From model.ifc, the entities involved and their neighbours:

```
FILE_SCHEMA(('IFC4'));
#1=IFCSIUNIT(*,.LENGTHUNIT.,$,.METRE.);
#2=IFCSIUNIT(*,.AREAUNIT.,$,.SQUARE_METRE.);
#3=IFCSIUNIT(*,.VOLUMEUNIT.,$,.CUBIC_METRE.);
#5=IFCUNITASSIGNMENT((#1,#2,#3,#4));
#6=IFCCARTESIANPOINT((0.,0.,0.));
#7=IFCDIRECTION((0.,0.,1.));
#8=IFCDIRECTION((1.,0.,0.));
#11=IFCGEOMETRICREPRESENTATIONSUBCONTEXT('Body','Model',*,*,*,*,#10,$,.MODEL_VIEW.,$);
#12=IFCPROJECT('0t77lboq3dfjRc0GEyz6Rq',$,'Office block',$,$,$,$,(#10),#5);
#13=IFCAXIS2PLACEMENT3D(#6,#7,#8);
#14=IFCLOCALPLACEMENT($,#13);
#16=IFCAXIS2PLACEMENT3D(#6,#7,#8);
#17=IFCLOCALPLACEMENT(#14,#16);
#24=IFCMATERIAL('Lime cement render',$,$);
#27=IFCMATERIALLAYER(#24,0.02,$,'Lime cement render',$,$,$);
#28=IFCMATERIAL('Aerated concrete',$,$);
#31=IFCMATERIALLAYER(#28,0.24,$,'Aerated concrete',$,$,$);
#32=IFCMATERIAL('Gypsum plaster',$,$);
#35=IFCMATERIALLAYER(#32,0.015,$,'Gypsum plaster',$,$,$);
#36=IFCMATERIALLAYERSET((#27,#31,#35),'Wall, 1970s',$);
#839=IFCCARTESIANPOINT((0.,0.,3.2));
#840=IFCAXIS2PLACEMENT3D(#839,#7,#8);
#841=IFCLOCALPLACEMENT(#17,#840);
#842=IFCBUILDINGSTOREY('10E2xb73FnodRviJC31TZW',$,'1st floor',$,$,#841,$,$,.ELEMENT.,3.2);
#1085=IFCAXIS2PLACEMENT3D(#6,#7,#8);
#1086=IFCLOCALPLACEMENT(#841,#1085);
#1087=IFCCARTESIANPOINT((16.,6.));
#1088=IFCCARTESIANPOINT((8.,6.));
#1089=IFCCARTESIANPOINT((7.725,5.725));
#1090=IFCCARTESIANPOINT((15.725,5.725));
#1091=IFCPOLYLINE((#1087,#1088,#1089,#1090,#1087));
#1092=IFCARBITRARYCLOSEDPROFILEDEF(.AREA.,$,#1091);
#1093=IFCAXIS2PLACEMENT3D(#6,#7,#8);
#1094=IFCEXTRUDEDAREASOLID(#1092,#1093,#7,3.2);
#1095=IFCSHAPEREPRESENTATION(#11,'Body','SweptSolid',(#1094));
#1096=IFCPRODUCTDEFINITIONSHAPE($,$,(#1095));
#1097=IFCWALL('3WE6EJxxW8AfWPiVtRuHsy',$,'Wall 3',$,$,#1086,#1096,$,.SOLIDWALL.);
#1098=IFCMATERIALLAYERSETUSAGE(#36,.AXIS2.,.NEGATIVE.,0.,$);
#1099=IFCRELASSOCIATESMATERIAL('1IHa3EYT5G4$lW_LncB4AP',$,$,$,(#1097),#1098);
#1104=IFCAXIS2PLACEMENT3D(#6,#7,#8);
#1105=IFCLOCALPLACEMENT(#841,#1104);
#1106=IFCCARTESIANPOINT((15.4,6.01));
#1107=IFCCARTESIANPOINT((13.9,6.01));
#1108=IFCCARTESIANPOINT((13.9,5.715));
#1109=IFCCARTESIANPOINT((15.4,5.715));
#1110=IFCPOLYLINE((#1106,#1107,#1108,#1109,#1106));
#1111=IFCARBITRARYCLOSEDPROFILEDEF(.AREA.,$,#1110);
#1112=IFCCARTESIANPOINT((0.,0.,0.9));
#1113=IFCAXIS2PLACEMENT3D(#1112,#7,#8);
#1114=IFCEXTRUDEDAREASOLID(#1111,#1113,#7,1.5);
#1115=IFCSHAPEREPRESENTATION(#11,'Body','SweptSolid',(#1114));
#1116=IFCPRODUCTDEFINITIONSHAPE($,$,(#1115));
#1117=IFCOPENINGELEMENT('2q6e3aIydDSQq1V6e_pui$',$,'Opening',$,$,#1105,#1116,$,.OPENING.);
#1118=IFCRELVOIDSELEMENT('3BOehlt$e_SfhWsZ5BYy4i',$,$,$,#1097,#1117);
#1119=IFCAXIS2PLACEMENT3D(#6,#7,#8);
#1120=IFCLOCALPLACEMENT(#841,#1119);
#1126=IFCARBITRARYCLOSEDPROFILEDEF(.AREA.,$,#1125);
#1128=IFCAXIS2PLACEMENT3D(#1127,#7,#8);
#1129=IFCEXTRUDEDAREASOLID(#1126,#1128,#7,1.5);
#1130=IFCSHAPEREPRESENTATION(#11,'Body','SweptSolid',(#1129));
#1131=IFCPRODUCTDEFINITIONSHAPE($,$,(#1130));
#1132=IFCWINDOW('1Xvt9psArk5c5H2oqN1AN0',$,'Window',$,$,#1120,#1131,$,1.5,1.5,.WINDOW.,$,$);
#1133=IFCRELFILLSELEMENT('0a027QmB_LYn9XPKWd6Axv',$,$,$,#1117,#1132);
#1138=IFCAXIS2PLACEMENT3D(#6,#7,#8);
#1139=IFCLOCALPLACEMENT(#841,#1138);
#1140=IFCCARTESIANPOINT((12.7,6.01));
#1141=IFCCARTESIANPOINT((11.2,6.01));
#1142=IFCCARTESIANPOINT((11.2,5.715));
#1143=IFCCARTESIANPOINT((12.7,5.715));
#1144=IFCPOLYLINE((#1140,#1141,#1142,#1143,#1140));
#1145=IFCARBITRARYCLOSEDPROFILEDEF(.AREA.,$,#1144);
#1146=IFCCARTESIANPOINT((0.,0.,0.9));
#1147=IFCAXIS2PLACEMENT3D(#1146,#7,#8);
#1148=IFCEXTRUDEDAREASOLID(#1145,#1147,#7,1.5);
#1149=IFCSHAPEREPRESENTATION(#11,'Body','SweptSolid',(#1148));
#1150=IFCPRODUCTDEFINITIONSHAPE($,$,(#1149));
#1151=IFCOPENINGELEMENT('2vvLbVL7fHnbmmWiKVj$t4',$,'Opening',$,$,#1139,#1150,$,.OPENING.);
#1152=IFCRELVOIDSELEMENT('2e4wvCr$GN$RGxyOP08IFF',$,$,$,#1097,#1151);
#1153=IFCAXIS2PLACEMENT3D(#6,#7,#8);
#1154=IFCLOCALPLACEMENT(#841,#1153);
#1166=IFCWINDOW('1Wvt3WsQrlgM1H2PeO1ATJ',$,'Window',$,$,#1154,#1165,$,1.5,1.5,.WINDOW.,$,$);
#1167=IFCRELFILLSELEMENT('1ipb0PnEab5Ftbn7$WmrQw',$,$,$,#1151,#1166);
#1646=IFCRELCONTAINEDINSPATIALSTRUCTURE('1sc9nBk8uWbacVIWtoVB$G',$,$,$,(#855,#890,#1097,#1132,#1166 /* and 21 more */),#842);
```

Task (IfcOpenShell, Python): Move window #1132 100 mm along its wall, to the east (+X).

```python
import ifcopenshell
import ifcopenshell.api.geometry
import ifcopenshell.util.placement
import ifcopenshell.util.unit

model = ifcopenshell.open("model.ifc")
unit_scale = ifcopenshell.util.unit.calculate_unit_scale(model)

window = model.by_id(1132)
opening = window.FillsVoids[0].RelatingOpeningElement
wall = opening.VoidsElements[0].RelatingBuildingElement

wall_matrix = ifcopenshell.util.placement.get_local_placement(wall.ObjectPlacement)
shift = wall_matrix[:3, 0] * 0.1 / unit_scale
before = ifcopenshell.util.placement.get_local_placement(window.ObjectPlacement)[:3, 3].copy()

# The window is not placed relative to its opening, so move both.
for product in (opening, window):
    matrix = ifcopenshell.util.placement.get_local_placement(product.ObjectPlacement)
    matrix[:3, 3] += shift
    ifcopenshell.api.geometry.edit_object_placement(model, product=product, matrix=matrix, is_si=False)

after = ifcopenshell.util.placement.get_local_placement(window.ObjectPlacement)[:3, 3]
print("window moved by", (after - before).round(3) + 0.0)

model.write("model_edited.ifc")
```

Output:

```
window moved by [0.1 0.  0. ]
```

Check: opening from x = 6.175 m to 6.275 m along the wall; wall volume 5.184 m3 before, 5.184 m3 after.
